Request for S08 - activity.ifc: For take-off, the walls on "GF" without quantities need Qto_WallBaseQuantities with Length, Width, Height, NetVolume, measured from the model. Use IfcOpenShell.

First a look at what the model holds.

```python
import ifcopenshell
import ifcopenshell.util.element
import ifcopenshell.util.unit

model = ifcopenshell.open("S08 - activity.ifc")
print(model.schema)
for unit_type in ("LENGTHUNIT", "AREAUNIT", "VOLUMEUNIT"):
    print(unit_type, ifcopenshell.util.unit.calculate_unit_scale(model, unit_type))
storey = next(s for s in model.by_type("IfcBuildingStorey") if s.Name == "GF")
walls = [e for e in ifcopenshell.util.element.get_decomposition(storey) if e.is_a("IfcWall")]
for e in sorted(walls, key=lambda e: e.id()):
    print(e.id(), e.is_a(), e.Name, list(ifcopenshell.util.element.get_psets(e, qtos_only=True)), sep=" | ")
```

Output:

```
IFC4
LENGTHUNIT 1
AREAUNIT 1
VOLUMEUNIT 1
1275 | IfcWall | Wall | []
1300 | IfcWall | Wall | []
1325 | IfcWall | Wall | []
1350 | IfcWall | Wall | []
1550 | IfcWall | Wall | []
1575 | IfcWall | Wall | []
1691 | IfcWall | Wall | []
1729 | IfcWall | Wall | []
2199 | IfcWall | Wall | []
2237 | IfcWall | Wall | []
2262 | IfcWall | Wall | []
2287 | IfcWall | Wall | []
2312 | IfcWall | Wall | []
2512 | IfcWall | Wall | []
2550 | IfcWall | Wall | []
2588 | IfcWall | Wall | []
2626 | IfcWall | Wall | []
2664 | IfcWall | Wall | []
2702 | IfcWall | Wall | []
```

```python
import ifcopenshell
import ifcopenshell.api.pset
import ifcopenshell.geom
import ifcopenshell.util.element
import ifcopenshell.util.shape
import ifcopenshell.util.unit

model = ifcopenshell.open("S08 - activity.ifc")
unit_scale = ifcopenshell.util.unit.calculate_unit_scale(model)
volume_scale = ifcopenshell.util.unit.calculate_unit_scale(model, "VOLUMEUNIT")
settings = ifcopenshell.geom.settings()

storey = next(s for s in model.by_type("IfcBuildingStorey") if s.Name == "GF")
walls = [e for e in ifcopenshell.util.element.get_decomposition(storey) if e.is_a("IfcWall")]

for e in sorted(walls, key=lambda e: e.id()):
    if ifcopenshell.util.element.get_psets(e, qtos_only=True, should_inherit=False):
        continue
    # Geometry comes back in metres, in the element's own axes.
    shape = ifcopenshell.geom.create_shape(settings, e)
    values = {
        "Length": ifcopenshell.util.shape.get_x(shape.geometry) / unit_scale,
        "Width": ifcopenshell.util.shape.get_y(shape.geometry) / unit_scale,
        "Height": ifcopenshell.util.shape.get_z(shape.geometry) / unit_scale,
        "NetVolume": ifcopenshell.util.shape.get_volume(shape.geometry) / volume_scale,
    }
    qto = ifcopenshell.api.pset.add_qto(model, product=e, name="Qto_WallBaseQuantities")
    ifcopenshell.api.pset.edit_qto(model, qto=qto, properties=values)
    print(e.id(), {k: round(v, 3) for k, v in values.items()})

model.write("S08 - activity_edited.ifc")
```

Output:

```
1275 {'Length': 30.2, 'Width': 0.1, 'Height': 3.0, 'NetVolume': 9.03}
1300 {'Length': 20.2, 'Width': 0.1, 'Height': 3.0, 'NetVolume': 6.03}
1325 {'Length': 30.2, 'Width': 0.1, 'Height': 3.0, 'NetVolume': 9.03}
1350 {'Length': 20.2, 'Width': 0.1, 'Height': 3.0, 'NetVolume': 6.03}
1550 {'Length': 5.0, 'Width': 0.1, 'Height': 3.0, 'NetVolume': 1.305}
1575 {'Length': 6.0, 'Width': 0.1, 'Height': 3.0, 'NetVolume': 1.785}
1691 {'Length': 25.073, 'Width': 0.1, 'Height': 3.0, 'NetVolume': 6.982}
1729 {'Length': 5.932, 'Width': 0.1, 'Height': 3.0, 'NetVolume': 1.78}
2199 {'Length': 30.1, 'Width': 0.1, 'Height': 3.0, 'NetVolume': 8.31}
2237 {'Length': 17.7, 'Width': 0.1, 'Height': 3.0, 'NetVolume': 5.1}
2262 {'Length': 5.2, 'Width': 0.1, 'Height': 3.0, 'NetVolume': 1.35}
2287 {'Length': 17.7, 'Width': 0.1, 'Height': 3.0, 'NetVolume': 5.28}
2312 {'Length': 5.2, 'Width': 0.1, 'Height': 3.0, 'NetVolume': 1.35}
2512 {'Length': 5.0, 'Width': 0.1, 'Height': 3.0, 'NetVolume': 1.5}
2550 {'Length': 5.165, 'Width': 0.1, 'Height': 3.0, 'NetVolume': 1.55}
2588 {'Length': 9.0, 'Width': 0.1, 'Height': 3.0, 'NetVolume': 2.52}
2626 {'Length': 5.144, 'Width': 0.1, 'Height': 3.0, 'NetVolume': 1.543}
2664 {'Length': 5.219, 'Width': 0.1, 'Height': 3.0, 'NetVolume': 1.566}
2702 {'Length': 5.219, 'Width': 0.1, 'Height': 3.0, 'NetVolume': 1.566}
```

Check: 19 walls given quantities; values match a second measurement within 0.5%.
